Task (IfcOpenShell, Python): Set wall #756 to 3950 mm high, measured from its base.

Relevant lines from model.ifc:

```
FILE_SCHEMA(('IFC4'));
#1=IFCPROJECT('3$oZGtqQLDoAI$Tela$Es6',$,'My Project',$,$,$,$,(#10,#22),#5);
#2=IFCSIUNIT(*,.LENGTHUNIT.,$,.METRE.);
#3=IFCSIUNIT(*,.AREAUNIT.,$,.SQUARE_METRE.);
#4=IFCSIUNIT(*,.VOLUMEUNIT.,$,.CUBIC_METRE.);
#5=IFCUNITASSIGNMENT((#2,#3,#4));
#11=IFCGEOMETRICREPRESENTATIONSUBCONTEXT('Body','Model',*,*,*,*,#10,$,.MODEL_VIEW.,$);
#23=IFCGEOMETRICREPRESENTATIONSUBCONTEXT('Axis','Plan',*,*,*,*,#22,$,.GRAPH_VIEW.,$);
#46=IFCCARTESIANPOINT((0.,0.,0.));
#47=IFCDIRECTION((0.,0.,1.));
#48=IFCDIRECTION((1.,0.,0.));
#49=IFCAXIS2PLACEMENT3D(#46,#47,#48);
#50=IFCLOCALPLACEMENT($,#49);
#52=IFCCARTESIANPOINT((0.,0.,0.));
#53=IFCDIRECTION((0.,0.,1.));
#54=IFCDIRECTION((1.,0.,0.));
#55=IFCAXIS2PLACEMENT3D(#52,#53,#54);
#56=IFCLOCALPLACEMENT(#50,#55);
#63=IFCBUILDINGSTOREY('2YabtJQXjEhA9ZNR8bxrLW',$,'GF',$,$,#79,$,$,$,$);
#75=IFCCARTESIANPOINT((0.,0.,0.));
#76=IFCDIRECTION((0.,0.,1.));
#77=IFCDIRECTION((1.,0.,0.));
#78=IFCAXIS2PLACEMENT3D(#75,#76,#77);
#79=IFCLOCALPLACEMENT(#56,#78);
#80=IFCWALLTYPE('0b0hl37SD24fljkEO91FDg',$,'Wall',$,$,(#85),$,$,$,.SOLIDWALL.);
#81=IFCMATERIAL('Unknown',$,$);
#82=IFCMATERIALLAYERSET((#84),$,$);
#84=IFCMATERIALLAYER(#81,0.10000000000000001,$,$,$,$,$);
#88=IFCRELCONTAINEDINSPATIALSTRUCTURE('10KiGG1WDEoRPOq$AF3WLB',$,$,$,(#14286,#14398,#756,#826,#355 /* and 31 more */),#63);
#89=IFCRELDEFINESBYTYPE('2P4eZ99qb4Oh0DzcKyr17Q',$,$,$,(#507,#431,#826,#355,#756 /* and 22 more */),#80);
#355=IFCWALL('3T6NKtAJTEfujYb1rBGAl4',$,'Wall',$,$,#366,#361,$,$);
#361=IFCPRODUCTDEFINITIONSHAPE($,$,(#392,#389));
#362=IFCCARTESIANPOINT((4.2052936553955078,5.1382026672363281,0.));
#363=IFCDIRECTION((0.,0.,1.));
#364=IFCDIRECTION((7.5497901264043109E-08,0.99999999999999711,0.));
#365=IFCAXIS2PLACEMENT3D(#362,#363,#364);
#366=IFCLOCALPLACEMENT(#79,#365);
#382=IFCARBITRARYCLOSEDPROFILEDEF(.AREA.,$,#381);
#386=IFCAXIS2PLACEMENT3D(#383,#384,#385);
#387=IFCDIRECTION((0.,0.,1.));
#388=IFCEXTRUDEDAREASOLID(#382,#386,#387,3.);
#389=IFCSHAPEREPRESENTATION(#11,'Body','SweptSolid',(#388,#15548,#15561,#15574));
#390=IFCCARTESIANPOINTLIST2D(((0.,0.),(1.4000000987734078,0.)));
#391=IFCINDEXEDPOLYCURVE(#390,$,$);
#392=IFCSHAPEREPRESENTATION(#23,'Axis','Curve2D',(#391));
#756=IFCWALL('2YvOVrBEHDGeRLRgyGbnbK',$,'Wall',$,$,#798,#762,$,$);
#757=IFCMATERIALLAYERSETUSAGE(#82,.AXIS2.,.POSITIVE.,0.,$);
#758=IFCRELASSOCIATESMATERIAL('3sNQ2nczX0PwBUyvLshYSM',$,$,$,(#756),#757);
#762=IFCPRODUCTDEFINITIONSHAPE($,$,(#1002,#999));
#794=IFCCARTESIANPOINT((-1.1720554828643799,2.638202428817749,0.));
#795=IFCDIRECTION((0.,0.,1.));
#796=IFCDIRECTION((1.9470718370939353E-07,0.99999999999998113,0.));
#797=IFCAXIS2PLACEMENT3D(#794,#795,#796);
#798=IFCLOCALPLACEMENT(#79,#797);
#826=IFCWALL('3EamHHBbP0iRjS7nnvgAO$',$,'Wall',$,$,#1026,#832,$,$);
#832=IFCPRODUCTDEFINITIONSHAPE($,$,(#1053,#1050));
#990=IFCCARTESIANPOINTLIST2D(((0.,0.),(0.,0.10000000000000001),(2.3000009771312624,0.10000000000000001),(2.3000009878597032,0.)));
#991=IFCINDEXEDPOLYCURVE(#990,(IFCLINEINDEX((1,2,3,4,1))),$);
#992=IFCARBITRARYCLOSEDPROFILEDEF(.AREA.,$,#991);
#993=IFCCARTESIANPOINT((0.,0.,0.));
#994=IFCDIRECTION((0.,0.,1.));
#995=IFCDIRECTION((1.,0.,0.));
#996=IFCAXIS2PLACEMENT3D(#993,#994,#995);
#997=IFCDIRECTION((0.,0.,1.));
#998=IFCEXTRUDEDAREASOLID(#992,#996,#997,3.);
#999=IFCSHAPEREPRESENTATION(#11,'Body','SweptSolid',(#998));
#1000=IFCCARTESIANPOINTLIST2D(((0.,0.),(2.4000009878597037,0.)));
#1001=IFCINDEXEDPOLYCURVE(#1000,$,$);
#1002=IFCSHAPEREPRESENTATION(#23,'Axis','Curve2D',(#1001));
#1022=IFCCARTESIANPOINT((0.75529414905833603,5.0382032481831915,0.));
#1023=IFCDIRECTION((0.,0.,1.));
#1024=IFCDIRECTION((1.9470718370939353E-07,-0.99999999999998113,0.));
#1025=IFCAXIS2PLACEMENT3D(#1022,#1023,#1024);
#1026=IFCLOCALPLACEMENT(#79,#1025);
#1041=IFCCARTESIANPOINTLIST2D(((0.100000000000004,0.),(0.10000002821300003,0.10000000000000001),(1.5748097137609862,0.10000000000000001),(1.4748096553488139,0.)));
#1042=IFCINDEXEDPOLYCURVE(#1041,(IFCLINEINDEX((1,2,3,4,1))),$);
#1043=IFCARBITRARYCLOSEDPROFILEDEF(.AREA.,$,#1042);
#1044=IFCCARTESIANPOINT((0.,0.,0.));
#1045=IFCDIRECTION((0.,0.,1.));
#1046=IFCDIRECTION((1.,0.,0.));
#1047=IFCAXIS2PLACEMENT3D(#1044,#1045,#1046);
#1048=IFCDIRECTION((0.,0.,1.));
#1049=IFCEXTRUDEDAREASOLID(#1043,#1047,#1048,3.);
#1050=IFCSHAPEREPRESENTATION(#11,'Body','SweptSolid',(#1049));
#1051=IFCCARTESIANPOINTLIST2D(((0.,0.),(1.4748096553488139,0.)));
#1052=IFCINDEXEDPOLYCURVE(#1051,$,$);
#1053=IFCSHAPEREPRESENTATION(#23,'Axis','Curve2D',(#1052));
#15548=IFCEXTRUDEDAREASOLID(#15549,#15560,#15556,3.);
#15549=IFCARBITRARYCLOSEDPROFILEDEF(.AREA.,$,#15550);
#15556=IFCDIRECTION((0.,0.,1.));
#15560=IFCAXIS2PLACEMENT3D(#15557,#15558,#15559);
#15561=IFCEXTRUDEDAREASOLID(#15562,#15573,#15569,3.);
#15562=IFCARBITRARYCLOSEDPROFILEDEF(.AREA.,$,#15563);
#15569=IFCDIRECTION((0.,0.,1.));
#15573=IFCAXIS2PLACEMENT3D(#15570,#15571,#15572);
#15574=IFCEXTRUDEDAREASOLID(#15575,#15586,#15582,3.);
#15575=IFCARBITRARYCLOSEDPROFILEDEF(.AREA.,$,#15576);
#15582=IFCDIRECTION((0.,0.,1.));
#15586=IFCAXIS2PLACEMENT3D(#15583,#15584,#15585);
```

```python
import ifcopenshell
import ifcopenshell.geom
import ifcopenshell.util.representation
import ifcopenshell.util.shape

model = ifcopenshell.open("model.ifc")
settings = ifcopenshell.geom.settings()


def volume(element):
    """Net volume in cubic metres, openings subtracted."""
    shape = ifcopenshell.geom.create_shape(settings, element)
    return ifcopenshell.util.shape.get_volume(shape.geometry)


wall = model.by_guid("2YvOVrBEHDGeRLRgyGbnbK")
before = volume(wall)

body = ifcopenshell.util.representation.get_representation(wall, "Model", "Body")
solid = body.Items[0]
old_height = solid.Depth
solid.Depth = 3.95
after = volume(wall)

print(f"height {old_height:g} -> {solid.Depth:g}, volume {before:.3f} -> {after:.3f} m3")

model.write("model_updated.ifc")
```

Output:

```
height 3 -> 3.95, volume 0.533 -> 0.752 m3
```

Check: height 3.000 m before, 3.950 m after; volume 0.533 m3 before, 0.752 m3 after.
